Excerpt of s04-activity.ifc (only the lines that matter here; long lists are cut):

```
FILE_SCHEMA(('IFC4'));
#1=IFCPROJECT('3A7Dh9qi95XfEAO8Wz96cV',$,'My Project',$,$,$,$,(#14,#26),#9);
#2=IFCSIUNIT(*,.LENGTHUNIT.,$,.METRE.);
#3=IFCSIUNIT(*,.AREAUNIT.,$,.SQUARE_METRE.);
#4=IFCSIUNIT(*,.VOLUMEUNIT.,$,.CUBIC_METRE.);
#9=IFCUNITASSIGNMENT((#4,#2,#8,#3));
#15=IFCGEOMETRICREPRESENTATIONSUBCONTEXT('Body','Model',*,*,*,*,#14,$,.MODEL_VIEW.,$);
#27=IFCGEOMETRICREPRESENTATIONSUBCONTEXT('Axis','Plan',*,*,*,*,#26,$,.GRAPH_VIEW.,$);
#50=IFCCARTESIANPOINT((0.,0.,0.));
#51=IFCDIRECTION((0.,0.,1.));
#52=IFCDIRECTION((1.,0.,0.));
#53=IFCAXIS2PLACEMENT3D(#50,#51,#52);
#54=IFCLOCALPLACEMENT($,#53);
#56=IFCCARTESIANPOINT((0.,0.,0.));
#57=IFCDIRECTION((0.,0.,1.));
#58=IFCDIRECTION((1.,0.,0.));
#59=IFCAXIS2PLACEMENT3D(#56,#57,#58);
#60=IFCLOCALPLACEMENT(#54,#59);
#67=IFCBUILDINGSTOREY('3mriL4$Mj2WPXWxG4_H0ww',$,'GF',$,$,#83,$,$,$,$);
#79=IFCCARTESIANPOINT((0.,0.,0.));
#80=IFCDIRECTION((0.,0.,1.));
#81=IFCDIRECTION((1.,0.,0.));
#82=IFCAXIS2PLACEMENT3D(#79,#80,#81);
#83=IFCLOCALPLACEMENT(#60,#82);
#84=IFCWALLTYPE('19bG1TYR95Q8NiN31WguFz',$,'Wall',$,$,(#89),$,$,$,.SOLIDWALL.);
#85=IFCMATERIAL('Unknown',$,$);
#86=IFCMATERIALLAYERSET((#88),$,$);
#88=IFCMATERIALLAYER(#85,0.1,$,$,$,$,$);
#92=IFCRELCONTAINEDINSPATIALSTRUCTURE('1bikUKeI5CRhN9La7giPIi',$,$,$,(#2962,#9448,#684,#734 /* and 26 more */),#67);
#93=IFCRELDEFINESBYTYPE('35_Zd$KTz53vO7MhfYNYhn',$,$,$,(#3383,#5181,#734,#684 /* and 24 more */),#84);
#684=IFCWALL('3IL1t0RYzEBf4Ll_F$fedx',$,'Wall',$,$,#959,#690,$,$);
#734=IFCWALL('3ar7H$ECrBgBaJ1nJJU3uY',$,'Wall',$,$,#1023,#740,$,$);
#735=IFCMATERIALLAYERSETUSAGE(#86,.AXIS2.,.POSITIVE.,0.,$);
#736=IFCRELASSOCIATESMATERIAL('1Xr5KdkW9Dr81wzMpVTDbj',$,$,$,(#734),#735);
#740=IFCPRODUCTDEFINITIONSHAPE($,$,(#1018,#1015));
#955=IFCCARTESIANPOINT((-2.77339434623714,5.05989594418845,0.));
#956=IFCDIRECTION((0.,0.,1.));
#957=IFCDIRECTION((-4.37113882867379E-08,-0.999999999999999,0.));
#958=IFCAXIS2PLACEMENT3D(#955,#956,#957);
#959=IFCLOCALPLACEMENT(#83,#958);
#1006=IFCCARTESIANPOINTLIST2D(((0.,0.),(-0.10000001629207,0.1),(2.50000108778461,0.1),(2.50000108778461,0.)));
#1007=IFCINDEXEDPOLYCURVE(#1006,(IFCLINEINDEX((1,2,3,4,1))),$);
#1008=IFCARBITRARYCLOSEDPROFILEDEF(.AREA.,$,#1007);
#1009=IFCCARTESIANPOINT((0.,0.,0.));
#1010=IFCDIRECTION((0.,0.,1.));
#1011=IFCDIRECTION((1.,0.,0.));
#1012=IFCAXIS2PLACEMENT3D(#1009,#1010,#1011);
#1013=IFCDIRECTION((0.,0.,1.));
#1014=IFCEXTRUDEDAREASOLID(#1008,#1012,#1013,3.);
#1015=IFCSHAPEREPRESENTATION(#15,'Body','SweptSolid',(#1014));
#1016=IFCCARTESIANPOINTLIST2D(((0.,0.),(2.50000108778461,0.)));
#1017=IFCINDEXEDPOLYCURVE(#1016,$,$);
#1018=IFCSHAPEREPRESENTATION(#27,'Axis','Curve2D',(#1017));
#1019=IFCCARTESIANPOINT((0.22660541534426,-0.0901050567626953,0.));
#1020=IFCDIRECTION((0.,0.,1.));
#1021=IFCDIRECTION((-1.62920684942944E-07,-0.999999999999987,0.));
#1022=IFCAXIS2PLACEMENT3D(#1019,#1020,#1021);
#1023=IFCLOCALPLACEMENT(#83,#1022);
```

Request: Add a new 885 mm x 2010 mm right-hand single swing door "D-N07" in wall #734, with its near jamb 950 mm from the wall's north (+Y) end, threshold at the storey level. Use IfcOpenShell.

```python
import numpy as np
import ifcopenshell
import ifcopenshell.api.feature
import ifcopenshell.api.geometry
import ifcopenshell.api.root
import ifcopenshell.api.spatial
import ifcopenshell.geom
import ifcopenshell.util.element
import ifcopenshell.util.placement
import ifcopenshell.util.representation
import ifcopenshell.util.shape
import ifcopenshell.util.unit

model = ifcopenshell.open("s04-activity.ifc")
unit_scale = ifcopenshell.util.unit.calculate_unit_scale(model)
settings = ifcopenshell.geom.settings()


def volume(element):
    """Net volume in cubic metres, openings subtracted."""
    shape = ifcopenshell.geom.create_shape(settings, element)
    return ifcopenshell.util.shape.get_volume(shape.geometry)


wall = model.by_guid("3ar7H$ECrBgBaJ1nJJU3uY")
storey = ifcopenshell.util.element.get_container(wall, ifc_class="IfcBuildingStorey")
context = ifcopenshell.util.representation.get_context(model, "Model", "Body", "MODEL_VIEW")
before = volume(wall)

width, height, from_end, sill = 0.885, 2.01, 0.95, 0.0  # metres

# The wall runs along its own X axis, and the end named is its -X end.
wall_shape = ifcopenshell.geom.create_shape(settings, wall)
x, y, z = ifcopenshell.util.shape.get_vertices(wall_shape.geometry).T
start = x.min() + from_end
face, thickness = float(y.min()), float(y.max() - y.min())
wall_matrix = ifcopenshell.util.placement.get_local_placement(wall.ObjectPlacement)
level = ifcopenshell.util.placement.get_local_placement(storey.ObjectPlacement)[2, 3]


def in_wall(x, y):
    """Placement at x, y metres in the wall's axes, at sill height."""
    matrix = wall_matrix.copy()
    matrix[:, 3] = wall_matrix @ np.array([x / unit_scale, y / unit_scale, 0.0, 1.0])
    matrix[2, 3] = level + sill / unit_scale
    return matrix


# Opening: a box that overshoots both wall faces by 50 mm.
opening = ifcopenshell.api.root.create_entity(model, ifc_class="IfcOpeningElement", predefined_type="OPENING")
box = ifcopenshell.api.geometry.add_wall_representation(
    model, context=context, length=width, height=height, thickness=thickness + 0.1
)
ifcopenshell.api.geometry.assign_representation(model, product=opening, representation=box)
ifcopenshell.api.geometry.edit_object_placement(model, product=opening, matrix=in_wall(start, face - 0.05), is_si=False)
ifcopenshell.api.feature.add_feature(model, feature=opening, element=wall)

door = ifcopenshell.api.root.create_entity(model, ifc_class="IfcDoor", name="D-N07", predefined_type="DOOR")
door.OverallWidth, door.OverallHeight = width / unit_scale, height / unit_scale
door.OperationType = "SINGLE_SWING_RIGHT"
body = ifcopenshell.api.geometry.add_door_representation(
    model,
    context=context,
    overall_width=door.OverallWidth,
    overall_height=door.OverallHeight,
    operation_type="SINGLE_SWING_RIGHT",
    lining_properties={"LiningDepth": thickness / unit_scale, "ThresholdDepth": thickness / unit_scale},
)
ifcopenshell.api.geometry.assign_representation(model, product=door, representation=body)
ifcopenshell.api.spatial.assign_container(model, products=[door], relating_structure=storey)
ifcopenshell.api.feature.add_filling(model, opening=opening, element=door)

# The lining spans the wall, so the door starts at the wall face.
ifcopenshell.api.geometry.edit_object_placement(model, product=door, matrix=in_wall(start, face), is_si=False)

after = volume(wall)

print(f"wall volume {before:.3f} -> {after:.3f} m3")

model.write("s04-activity_v2.ifc")
```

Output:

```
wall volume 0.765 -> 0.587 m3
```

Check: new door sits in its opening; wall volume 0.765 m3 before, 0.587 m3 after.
